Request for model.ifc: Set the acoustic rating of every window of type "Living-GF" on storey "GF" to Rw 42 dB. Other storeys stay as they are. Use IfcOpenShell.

First a look at what the model holds.

```python
import ifcopenshell
import ifcopenshell.util.element

model = ifcopenshell.open("model.ifc")
print(model.schema)
storey = next(s for s in model.by_type("IfcBuildingStorey") if s.Name == "GF")
windows = [e for e in ifcopenshell.util.element.get_decomposition(storey) if e.is_a("IfcWindow")]
seen = {}
for e in windows:
    element_type = ifcopenshell.util.element.get_type(e)
    key = (element_type.Name if element_type != e and element_type else None, ifcopenshell.util.element.get_pset(e, "Pset_WindowCommon", "AcousticRating"))
    seen[key] = seen.get(key, 0) + 1
for (name, value), count in sorted(seen.items(), key=str):
    print(count, "x", name, "|", value)
```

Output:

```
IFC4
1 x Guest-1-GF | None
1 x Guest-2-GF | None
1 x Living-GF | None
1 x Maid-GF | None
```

```python
import ifcopenshell
import ifcopenshell.api.pset
import ifcopenshell.util.element

model = ifcopenshell.open("model.ifc")

storey = next(s for s in model.by_type("IfcBuildingStorey") if s.Name == "GF")
windows = [e for e in ifcopenshell.util.element.get_decomposition(storey) if e.is_a("IfcWindow")]

count = 0
for e in windows:
    element_type = ifcopenshell.util.element.get_type(e)
    if element_type in (None, e) or element_type.Name != "Living-GF":
        continue
    # add_pset returns the element's existing set when there is one.
    pset = ifcopenshell.api.pset.add_pset(model, product=e, name="Pset_WindowCommon")
    ifcopenshell.api.pset.edit_pset(model, pset=pset, properties={"AcousticRating": "Rw 42 dB"})
    count += 1

print(count, "windows updated")

model.write("model_edited.ifc")
```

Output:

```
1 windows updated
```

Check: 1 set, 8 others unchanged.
